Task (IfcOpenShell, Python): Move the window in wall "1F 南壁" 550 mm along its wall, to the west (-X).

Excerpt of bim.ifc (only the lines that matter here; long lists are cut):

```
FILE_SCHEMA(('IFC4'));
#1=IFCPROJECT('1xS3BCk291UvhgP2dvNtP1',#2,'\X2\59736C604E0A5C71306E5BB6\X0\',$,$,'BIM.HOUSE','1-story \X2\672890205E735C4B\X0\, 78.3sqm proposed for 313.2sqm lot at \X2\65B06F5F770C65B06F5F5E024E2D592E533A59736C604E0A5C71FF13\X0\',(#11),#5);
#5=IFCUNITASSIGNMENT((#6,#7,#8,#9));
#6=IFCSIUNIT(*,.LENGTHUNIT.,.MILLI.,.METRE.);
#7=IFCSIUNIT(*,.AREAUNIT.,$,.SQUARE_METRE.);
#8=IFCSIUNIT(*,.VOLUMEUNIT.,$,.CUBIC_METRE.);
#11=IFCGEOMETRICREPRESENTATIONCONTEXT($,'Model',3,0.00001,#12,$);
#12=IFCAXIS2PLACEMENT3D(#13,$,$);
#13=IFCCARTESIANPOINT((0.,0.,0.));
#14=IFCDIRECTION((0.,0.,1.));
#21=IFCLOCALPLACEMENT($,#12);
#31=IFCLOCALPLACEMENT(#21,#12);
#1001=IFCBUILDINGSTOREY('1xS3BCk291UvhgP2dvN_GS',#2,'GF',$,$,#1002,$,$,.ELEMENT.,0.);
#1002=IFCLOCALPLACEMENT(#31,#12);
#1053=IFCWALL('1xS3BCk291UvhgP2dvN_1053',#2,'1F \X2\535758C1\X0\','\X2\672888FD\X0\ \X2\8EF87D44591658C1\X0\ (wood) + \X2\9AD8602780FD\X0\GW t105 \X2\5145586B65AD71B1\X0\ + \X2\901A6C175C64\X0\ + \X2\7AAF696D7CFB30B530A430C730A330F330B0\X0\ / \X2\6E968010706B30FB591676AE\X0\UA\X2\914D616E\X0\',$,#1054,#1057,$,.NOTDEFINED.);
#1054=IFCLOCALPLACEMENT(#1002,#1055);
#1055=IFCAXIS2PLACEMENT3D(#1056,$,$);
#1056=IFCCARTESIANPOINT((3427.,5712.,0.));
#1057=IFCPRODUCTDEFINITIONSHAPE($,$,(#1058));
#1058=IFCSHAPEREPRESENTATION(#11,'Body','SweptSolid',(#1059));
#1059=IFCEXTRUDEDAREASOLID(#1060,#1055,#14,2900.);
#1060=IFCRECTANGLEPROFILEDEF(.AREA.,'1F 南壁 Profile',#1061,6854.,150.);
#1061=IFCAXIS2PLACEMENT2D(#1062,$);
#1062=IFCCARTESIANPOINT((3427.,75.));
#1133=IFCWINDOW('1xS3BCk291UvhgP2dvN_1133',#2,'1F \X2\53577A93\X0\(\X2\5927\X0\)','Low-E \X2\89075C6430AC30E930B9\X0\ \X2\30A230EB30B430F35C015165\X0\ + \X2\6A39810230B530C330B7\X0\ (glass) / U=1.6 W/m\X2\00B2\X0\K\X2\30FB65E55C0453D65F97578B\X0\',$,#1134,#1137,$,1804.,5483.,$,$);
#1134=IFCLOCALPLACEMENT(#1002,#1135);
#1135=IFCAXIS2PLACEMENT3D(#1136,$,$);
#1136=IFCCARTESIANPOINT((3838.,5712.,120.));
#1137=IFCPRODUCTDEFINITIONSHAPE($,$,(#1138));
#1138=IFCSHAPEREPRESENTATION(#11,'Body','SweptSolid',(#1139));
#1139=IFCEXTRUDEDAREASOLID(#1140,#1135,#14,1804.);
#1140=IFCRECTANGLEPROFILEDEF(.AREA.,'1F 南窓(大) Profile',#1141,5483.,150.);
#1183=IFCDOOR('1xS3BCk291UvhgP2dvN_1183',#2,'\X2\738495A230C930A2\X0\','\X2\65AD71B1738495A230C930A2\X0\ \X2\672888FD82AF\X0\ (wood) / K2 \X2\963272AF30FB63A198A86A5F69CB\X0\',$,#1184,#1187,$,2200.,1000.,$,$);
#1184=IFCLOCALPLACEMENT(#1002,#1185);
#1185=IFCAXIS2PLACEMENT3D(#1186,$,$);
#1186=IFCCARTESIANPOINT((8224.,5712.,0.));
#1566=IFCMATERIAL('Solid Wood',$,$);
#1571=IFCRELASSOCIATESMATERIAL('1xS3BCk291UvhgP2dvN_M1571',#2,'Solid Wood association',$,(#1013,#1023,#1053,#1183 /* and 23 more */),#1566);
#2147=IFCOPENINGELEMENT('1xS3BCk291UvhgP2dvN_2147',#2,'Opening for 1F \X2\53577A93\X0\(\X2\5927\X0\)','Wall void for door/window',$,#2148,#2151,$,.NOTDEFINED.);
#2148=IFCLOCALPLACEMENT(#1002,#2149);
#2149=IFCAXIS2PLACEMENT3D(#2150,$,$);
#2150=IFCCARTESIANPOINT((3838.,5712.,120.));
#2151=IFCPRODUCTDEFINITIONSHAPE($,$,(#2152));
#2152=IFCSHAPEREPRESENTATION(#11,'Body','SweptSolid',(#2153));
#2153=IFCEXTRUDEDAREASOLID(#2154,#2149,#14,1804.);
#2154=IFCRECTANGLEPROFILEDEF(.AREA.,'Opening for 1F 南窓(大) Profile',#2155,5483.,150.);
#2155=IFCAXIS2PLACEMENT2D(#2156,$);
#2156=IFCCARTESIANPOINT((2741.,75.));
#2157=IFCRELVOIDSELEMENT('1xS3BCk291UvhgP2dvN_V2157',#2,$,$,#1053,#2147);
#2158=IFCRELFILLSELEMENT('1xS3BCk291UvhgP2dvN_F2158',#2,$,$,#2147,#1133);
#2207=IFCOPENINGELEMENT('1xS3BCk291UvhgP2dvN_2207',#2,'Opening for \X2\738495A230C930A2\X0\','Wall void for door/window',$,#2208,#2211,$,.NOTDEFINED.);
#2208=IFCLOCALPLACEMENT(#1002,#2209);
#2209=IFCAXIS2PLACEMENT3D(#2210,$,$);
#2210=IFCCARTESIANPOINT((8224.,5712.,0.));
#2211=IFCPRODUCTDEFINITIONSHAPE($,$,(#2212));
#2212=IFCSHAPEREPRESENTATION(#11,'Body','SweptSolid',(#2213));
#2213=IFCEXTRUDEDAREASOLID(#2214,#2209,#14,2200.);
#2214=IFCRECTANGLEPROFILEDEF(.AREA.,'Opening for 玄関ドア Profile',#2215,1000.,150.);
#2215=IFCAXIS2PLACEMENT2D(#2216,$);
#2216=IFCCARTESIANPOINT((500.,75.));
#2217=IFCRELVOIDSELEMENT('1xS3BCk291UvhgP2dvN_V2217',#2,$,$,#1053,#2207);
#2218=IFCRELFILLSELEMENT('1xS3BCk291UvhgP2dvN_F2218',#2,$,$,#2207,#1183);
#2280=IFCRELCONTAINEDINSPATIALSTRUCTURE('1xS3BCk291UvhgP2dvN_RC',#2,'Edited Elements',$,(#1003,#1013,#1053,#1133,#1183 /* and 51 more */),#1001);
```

```python
import ifcopenshell
import ifcopenshell.api.geometry
import ifcopenshell.util.placement

model = ifcopenshell.open("bim.ifc")

window = model.by_id(1133)
opening = window.FillsVoids[0].RelatingOpeningElement
wall = opening.VoidsElements[0].RelatingBuildingElement

wall_matrix = ifcopenshell.util.placement.get_local_placement(wall.ObjectPlacement)
shift = wall_matrix[:3, 0] * -550.0
before = ifcopenshell.util.placement.get_local_placement(window.ObjectPlacement)[:3, 3].copy()

# The window is not placed relative to its opening, so move both.
for product in (opening, window):
    matrix = ifcopenshell.util.placement.get_local_placement(product.ObjectPlacement)
    matrix[:3, 3] += shift
    ifcopenshell.api.geometry.edit_object_placement(model, product=product, matrix=matrix, is_si=False)

after = ifcopenshell.util.placement.get_local_placement(window.ObjectPlacement)[:3, 3]
print("window moved by", (after - before).round(3) + 0.0)

model.write("bim_v2.ifc")
```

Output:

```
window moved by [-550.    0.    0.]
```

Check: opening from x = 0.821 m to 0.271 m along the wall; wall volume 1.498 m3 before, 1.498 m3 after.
